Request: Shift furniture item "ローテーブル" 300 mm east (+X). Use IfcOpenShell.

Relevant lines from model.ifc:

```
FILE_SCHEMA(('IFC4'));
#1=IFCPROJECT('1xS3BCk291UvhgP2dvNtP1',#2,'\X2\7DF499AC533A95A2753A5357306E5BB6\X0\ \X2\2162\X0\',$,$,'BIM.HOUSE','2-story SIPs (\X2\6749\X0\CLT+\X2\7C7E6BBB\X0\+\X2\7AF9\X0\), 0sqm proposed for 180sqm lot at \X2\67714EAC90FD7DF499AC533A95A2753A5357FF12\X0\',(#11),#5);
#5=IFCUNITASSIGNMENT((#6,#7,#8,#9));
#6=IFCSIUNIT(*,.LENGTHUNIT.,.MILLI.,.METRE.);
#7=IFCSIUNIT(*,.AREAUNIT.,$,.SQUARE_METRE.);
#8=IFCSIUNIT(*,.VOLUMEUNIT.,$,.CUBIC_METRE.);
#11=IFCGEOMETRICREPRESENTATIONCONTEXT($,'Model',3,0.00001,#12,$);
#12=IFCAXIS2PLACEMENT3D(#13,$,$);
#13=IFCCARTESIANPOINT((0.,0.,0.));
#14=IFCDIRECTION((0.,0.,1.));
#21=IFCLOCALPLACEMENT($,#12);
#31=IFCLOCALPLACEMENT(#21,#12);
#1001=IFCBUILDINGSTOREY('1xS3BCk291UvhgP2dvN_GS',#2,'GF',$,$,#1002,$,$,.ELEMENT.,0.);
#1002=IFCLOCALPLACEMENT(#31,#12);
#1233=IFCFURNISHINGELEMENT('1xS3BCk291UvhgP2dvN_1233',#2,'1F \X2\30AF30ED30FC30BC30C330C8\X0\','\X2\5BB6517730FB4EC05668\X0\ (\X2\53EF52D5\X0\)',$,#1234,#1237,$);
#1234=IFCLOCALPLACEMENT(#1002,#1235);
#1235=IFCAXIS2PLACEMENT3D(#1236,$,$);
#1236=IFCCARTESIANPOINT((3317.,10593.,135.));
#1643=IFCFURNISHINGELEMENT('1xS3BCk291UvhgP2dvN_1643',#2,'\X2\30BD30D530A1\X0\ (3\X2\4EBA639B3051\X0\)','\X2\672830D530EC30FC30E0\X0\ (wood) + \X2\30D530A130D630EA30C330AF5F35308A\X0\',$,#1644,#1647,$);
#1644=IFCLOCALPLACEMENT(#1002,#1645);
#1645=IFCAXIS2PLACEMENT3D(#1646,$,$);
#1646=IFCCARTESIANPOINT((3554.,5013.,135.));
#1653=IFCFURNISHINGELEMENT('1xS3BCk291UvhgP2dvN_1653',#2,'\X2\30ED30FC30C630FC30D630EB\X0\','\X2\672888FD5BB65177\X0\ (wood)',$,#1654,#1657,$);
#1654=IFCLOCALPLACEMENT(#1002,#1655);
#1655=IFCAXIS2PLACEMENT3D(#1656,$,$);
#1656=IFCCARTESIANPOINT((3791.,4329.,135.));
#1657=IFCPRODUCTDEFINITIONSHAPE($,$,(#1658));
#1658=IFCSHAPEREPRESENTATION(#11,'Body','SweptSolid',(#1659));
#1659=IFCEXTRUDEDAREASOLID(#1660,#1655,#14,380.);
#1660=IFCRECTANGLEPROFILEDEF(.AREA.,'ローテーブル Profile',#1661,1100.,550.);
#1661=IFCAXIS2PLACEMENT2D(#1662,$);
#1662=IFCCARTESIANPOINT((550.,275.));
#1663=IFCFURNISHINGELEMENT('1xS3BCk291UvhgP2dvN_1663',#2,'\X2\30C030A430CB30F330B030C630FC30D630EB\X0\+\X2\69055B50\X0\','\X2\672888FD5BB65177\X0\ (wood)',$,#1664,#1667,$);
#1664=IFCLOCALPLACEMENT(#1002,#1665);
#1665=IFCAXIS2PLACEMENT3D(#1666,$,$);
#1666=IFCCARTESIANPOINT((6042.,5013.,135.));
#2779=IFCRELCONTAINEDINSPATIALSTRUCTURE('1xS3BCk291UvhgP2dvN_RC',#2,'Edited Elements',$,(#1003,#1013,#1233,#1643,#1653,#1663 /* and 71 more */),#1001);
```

```python
import ifcopenshell
import ifcopenshell.api.geometry
import ifcopenshell.util.placement

model = ifcopenshell.open("model.ifc")

item = model.by_guid("1xS3BCk291UvhgP2dvN_1653")
matrix = ifcopenshell.util.placement.get_local_placement(item.ObjectPlacement)
matrix[0, 3] += 300.0
ifcopenshell.api.geometry.edit_object_placement(model, product=item, matrix=matrix, is_si=False)

print(ifcopenshell.util.placement.get_local_placement(item.ObjectPlacement).round(3) + 0.0)

model.write("model_edited.ifc")
```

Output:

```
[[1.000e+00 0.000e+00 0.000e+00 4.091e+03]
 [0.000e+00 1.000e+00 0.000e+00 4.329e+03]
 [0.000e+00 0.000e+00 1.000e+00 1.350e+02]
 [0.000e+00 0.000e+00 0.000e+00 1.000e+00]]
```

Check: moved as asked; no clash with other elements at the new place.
